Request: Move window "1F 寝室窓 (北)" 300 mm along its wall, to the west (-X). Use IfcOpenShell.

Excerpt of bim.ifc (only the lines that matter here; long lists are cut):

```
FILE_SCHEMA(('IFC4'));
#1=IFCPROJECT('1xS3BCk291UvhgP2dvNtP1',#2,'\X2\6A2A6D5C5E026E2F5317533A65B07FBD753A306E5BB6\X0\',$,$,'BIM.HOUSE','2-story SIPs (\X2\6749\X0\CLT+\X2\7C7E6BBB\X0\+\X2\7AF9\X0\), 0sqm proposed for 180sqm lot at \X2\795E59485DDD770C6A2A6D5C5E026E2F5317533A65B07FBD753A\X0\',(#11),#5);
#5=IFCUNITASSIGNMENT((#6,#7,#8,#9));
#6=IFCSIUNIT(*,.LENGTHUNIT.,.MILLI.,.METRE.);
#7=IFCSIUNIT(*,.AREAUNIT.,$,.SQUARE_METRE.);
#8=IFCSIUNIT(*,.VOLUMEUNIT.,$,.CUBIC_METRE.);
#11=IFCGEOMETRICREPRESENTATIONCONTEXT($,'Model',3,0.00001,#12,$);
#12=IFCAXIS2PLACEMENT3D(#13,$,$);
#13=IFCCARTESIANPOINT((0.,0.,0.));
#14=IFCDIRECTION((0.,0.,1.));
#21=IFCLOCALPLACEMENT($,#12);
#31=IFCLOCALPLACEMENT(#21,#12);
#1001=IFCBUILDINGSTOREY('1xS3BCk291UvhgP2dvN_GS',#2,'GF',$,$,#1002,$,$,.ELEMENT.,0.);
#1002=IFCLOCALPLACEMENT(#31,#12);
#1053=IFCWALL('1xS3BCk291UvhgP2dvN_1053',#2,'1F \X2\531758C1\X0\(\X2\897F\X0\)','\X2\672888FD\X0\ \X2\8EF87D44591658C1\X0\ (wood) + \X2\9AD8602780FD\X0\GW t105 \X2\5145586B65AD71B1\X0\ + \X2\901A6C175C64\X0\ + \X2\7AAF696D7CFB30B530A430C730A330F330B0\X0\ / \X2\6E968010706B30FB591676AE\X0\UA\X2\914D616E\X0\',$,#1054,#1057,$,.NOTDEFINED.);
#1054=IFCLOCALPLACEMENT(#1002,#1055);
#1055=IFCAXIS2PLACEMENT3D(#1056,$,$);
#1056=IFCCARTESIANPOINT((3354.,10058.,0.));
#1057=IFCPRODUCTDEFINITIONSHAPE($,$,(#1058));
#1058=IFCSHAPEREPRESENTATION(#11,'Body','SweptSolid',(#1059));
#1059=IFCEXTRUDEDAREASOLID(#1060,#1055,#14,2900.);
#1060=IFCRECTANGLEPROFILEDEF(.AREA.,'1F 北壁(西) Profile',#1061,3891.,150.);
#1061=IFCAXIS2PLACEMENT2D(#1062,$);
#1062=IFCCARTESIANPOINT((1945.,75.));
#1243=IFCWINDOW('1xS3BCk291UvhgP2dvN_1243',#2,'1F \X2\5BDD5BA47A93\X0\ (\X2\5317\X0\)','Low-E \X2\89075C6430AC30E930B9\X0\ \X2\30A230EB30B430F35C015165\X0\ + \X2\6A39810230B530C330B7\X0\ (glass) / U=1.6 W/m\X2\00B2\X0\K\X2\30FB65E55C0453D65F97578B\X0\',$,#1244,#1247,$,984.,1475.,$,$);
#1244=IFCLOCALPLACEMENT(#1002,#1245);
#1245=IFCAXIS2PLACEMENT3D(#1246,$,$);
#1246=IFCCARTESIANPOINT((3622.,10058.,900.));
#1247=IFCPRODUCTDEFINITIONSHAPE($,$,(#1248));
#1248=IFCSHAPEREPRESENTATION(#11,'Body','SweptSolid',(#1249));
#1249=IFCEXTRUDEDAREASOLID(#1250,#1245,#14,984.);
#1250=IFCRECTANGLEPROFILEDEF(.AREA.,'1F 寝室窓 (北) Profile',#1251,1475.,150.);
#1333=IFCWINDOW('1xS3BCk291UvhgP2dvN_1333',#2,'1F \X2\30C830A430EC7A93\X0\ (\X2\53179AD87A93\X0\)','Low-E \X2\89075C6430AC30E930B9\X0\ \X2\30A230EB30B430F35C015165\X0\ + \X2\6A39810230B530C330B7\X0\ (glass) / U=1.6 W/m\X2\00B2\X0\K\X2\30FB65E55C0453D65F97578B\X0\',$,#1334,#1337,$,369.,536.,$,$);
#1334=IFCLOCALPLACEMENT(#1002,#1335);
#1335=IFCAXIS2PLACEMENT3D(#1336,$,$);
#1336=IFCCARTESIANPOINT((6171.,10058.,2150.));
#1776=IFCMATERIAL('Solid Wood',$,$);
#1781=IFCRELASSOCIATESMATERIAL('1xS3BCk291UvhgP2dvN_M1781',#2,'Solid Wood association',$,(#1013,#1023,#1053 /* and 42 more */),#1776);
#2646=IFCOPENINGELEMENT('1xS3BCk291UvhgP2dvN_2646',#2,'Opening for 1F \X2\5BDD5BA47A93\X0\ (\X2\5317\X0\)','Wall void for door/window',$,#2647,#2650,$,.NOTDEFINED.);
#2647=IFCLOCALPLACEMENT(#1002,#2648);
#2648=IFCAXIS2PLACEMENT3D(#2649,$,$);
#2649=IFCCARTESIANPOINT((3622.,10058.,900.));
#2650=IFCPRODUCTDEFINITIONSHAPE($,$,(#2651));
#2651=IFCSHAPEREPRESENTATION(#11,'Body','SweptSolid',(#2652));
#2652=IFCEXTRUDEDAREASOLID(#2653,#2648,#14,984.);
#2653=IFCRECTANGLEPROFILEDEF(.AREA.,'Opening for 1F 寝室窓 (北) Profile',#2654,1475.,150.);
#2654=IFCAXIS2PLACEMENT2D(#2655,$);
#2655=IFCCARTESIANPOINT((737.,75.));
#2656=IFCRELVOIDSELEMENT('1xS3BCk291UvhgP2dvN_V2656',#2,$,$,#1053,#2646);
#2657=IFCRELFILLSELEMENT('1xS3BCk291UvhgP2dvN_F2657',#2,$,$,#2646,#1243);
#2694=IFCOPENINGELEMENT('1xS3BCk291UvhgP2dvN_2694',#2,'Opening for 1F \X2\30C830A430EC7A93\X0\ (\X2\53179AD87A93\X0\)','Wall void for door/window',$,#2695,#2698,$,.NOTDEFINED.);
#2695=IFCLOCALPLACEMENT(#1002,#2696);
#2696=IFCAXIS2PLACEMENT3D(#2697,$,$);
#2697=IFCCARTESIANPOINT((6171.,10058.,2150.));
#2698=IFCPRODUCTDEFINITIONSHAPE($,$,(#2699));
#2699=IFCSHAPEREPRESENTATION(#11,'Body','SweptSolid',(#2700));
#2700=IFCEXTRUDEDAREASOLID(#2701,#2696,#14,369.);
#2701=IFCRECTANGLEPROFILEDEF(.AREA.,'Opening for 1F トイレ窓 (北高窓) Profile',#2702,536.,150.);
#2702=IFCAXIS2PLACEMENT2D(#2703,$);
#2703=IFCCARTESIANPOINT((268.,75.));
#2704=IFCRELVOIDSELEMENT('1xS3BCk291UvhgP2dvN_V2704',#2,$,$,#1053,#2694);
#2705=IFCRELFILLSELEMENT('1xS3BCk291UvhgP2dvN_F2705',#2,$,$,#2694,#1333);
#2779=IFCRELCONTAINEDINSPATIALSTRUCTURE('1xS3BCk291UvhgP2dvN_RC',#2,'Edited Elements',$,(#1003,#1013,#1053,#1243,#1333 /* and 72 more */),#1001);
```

```python
import ifcopenshell
import ifcopenshell.api.geometry
import ifcopenshell.util.placement
import ifcopenshell.util.unit

model = ifcopenshell.open("bim.ifc")
unit_scale = ifcopenshell.util.unit.calculate_unit_scale(model)

window = model.by_guid("1xS3BCk291UvhgP2dvN_1243")
opening = window.FillsVoids[0].RelatingOpeningElement
wall = opening.VoidsElements[0].RelatingBuildingElement

wall_matrix = ifcopenshell.util.placement.get_local_placement(wall.ObjectPlacement)
shift = wall_matrix[:3, 0] * -0.3 / unit_scale
before = ifcopenshell.util.placement.get_local_placement(window.ObjectPlacement)[:3, 3].copy()

# The window is not placed relative to its opening, so move both.
for product in (opening, window):
    matrix = ifcopenshell.util.placement.get_local_placement(product.ObjectPlacement)
    matrix[:3, 3] += shift
    ifcopenshell.api.geometry.edit_object_placement(model, product=product, matrix=matrix, is_si=False)

after = ifcopenshell.util.placement.get_local_placement(window.ObjectPlacement)[:3, 3]
print("window moved by", (after - before).round(3) + 0.0)

model.write("bim_updated.ifc")
```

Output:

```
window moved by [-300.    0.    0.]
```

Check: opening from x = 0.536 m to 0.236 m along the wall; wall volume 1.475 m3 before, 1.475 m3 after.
